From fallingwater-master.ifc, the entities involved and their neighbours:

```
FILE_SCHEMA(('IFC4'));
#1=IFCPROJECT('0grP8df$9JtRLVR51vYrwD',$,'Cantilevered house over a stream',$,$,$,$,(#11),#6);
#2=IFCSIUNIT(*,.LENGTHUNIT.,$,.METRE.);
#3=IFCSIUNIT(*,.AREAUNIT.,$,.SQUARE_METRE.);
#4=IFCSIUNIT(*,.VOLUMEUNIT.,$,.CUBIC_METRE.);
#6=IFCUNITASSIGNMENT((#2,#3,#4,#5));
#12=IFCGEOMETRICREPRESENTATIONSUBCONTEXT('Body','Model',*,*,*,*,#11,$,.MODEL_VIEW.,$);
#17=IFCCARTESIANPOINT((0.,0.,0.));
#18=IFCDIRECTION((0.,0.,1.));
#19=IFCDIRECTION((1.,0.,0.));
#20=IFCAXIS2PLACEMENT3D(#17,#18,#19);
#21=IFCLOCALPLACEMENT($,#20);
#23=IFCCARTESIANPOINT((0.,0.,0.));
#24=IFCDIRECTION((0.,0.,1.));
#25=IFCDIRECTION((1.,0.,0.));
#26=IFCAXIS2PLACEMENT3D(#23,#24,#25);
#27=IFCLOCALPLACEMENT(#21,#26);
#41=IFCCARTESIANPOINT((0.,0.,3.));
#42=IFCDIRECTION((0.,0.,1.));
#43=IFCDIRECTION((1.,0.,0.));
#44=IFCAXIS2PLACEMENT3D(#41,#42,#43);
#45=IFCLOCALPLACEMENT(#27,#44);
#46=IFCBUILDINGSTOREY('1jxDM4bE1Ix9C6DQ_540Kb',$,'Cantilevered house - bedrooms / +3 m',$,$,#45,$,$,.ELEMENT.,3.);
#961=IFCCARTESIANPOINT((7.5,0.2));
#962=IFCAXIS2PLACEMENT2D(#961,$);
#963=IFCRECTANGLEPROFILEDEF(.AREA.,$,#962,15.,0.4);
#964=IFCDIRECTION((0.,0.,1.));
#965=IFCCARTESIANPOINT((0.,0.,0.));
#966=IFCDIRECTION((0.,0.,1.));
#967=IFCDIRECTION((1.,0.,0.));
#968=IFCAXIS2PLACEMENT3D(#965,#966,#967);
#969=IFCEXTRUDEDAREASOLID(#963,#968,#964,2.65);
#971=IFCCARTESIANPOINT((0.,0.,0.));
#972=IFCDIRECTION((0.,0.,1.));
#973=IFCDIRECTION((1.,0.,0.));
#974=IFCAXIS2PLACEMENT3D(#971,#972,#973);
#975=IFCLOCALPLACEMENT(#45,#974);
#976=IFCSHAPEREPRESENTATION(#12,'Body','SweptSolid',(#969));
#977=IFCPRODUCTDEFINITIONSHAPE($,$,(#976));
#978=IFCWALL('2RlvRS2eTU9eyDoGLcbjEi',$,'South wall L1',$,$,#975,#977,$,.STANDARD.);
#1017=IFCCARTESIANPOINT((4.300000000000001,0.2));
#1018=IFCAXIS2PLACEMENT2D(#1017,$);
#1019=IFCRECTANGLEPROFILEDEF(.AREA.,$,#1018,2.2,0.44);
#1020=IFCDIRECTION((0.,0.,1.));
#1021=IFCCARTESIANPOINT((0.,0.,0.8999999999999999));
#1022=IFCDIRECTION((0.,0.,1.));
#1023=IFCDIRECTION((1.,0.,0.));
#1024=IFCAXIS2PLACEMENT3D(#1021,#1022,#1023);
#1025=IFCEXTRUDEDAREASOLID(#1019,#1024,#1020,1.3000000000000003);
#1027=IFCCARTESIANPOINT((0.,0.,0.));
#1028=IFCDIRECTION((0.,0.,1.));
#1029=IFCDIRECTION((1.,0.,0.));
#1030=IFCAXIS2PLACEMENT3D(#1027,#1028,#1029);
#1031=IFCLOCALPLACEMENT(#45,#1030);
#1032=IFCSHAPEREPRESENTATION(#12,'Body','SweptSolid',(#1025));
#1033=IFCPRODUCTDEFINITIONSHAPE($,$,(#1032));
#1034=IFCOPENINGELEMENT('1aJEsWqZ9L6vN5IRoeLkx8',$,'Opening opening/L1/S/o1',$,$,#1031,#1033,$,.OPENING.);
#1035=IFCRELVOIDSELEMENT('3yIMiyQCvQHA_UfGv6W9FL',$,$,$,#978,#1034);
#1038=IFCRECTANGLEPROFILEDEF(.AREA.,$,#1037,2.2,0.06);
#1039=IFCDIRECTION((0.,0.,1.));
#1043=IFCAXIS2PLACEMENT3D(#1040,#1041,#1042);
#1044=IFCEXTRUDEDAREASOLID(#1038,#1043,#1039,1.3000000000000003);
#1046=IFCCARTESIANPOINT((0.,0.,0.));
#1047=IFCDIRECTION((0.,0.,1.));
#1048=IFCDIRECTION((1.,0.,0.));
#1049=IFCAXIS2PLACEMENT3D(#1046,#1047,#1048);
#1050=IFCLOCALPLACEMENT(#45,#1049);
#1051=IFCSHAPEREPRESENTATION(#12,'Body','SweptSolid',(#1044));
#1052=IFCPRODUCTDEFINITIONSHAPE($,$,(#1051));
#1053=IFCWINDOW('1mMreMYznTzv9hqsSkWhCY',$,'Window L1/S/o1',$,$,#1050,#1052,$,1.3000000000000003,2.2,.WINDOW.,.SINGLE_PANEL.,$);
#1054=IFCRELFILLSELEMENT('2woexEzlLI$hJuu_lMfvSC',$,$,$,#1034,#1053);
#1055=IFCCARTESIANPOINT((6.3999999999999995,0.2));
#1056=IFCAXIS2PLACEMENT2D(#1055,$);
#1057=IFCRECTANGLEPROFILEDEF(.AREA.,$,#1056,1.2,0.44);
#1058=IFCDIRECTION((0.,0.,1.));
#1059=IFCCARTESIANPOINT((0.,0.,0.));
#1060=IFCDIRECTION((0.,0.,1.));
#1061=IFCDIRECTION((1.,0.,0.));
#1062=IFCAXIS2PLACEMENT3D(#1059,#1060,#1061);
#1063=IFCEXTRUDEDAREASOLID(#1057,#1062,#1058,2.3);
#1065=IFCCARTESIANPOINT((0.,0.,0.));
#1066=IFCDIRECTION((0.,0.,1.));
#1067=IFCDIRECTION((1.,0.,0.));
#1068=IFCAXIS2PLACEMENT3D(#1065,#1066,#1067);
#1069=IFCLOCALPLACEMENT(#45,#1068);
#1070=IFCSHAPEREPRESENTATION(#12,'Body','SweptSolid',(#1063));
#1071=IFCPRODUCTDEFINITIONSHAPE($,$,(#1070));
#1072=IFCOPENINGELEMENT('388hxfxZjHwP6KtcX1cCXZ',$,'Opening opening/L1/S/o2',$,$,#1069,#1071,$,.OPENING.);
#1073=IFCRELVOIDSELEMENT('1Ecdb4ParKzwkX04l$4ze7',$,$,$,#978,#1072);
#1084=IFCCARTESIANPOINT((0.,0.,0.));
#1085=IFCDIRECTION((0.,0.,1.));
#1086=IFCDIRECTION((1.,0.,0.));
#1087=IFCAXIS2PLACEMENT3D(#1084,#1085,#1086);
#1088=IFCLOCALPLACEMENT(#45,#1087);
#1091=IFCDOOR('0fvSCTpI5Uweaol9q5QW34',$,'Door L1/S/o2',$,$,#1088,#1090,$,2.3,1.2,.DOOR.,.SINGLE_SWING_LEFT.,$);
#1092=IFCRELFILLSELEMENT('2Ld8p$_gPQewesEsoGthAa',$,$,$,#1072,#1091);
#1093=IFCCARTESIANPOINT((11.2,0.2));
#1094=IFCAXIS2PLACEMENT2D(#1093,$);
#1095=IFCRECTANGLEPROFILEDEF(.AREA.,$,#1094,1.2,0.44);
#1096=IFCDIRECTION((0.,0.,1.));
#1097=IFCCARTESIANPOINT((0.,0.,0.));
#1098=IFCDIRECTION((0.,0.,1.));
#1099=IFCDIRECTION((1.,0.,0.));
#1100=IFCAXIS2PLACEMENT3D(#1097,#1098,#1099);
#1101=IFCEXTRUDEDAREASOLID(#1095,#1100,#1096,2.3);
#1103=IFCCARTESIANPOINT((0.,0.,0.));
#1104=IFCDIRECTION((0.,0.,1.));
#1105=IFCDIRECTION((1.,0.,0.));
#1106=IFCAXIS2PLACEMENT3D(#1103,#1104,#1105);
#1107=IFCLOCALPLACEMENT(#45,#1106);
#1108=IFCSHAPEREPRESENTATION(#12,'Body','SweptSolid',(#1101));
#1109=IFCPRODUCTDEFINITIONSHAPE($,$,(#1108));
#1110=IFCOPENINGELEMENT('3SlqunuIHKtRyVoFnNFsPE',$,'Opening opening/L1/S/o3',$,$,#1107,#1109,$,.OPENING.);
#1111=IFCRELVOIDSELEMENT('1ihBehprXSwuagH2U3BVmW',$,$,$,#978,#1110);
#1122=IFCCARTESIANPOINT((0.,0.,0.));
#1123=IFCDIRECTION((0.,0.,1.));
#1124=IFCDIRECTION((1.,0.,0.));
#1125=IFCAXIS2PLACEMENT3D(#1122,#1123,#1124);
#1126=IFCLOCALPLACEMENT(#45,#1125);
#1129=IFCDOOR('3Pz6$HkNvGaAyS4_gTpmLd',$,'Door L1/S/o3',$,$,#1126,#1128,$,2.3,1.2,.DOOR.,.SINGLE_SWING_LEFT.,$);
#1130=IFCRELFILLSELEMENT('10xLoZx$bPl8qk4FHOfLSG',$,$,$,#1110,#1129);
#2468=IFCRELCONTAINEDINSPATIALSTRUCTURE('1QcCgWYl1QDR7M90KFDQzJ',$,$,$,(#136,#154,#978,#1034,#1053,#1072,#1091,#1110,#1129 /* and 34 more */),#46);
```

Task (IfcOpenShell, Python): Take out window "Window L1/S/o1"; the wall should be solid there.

```python
import ifcopenshell
import ifcopenshell.api.feature
import ifcopenshell.api.root
import ifcopenshell.geom
import ifcopenshell.util.shape

model = ifcopenshell.open("fallingwater-master.ifc")
settings = ifcopenshell.geom.settings()


def volume(element):
    """Net volume in cubic metres, openings subtracted."""
    shape = ifcopenshell.geom.create_shape(settings, element)
    return ifcopenshell.util.shape.get_volume(shape.geometry)


window = model.by_id(1053)
opening = window.FillsVoids[0].RelatingOpeningElement
wall = opening.VoidsElements[0].RelatingBuildingElement
before = volume(wall)

ifcopenshell.api.root.remove_product(model, product=window)
ifcopenshell.api.feature.remove_feature(model, feature=opening)

after = volume(wall)

print(f"wall volume {before:.3f} -> {after:.3f} m3")

model.write("fallingwater-master_rev.ifc")
```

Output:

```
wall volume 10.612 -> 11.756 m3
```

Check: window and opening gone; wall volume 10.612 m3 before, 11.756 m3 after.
